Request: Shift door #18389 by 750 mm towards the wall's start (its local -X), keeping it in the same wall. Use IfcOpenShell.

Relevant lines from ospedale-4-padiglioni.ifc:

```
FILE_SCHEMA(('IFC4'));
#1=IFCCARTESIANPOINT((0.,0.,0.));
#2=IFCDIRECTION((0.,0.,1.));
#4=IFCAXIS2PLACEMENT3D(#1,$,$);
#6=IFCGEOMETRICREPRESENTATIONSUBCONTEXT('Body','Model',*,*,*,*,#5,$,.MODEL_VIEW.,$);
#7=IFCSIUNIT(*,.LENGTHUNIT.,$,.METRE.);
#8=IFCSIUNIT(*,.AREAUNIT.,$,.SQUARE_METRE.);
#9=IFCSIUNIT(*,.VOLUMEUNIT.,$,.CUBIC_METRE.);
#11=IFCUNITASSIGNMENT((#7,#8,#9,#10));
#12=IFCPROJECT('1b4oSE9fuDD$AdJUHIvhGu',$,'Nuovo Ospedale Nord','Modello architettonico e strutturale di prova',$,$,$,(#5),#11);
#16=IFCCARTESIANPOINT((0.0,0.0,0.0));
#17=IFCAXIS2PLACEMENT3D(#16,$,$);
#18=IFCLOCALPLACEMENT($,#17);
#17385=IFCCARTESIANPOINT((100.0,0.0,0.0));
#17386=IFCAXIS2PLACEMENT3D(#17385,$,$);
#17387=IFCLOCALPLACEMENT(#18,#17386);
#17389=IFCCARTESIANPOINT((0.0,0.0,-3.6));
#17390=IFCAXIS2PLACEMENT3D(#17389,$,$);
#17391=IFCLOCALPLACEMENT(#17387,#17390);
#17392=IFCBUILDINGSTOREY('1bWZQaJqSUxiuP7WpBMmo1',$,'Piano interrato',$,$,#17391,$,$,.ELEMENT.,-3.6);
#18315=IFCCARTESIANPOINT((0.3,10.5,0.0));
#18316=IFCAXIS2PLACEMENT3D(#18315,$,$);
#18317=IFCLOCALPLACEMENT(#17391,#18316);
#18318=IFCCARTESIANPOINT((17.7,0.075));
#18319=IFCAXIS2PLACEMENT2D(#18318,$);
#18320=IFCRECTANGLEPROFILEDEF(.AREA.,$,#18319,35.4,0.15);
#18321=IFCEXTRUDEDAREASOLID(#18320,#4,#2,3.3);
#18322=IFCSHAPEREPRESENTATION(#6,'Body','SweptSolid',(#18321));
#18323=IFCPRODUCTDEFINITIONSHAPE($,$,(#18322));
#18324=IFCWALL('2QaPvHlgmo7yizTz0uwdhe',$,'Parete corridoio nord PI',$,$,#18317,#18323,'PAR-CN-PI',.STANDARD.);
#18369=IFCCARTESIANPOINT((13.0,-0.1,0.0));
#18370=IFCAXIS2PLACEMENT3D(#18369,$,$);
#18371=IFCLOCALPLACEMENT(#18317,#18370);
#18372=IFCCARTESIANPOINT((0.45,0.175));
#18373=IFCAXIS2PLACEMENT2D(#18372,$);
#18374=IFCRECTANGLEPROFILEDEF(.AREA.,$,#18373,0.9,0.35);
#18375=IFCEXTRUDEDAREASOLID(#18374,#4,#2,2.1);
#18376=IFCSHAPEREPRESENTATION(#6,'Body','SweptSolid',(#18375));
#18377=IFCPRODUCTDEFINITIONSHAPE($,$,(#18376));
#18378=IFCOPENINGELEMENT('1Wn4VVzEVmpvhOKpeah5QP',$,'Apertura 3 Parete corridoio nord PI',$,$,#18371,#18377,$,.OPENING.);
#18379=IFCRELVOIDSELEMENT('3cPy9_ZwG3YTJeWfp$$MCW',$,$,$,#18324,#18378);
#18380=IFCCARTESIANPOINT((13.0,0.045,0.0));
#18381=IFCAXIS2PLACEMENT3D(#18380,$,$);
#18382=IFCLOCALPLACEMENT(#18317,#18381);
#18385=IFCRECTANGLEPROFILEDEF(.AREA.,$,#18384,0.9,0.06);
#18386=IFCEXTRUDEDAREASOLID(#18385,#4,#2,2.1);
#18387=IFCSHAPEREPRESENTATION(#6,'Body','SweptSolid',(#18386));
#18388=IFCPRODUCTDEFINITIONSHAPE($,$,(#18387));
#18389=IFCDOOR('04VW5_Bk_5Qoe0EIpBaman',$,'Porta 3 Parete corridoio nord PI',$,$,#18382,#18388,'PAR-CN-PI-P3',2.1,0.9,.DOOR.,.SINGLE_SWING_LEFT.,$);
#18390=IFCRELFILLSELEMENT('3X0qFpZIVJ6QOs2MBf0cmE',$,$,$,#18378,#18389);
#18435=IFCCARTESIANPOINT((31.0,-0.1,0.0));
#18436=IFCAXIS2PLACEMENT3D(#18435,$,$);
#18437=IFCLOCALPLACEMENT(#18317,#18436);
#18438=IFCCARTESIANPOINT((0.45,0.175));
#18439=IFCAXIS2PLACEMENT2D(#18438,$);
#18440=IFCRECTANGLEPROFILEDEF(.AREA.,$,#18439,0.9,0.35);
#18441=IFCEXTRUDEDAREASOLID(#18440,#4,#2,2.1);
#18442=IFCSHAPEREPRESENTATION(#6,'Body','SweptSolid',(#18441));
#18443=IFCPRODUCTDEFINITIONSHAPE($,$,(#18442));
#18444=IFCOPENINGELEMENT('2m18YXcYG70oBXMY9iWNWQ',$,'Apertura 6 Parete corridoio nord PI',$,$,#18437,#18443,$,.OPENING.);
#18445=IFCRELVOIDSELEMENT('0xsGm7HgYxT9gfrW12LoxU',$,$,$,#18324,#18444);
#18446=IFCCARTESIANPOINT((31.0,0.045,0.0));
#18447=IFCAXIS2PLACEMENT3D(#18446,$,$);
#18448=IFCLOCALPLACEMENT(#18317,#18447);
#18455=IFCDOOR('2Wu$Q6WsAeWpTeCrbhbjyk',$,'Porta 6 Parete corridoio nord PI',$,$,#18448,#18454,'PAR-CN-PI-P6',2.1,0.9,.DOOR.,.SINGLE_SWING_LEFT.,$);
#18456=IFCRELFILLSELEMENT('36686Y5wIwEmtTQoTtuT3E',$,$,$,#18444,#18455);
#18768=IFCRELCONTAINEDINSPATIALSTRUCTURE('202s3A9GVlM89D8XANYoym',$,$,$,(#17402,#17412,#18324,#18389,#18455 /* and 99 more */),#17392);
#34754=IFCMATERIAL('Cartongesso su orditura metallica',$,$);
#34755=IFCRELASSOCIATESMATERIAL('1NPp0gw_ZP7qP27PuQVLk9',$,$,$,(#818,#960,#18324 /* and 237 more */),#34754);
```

```python
import ifcopenshell
import ifcopenshell.api.geometry
import ifcopenshell.util.placement

model = ifcopenshell.open("ospedale-4-padiglioni.ifc")

door = model.by_guid("04VW5_Bk_5Qoe0EIpBaman")
opening = door.FillsVoids[0].RelatingOpeningElement
wall = opening.VoidsElements[0].RelatingBuildingElement

wall_matrix = ifcopenshell.util.placement.get_local_placement(wall.ObjectPlacement)
shift = wall_matrix[:3, 0] * -0.75
before = ifcopenshell.util.placement.get_local_placement(door.ObjectPlacement)[:3, 3].copy()

# The door is not placed relative to its opening, so move both.
for product in (opening, door):
    matrix = ifcopenshell.util.placement.get_local_placement(product.ObjectPlacement)
    matrix[:3, 3] += shift
    ifcopenshell.api.geometry.edit_object_placement(model, product=product, matrix=matrix, is_si=False)

after = ifcopenshell.util.placement.get_local_placement(door.ObjectPlacement)[:3, 3]
print("door moved by", (after - before).round(3) + 0.0)

model.write("ospedale-4-padiglioni_rev.ifc")
```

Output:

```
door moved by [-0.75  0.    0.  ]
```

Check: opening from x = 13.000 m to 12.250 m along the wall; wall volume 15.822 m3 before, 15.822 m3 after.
